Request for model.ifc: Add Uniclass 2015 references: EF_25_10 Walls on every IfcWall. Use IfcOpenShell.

First a look at what the model holds.

```python
import ifcopenshell

model = ifcopenshell.open("model.ifc")
print(model.schema)
print("classifications:", [c.Name for c in model.by_type("IfcClassification")])
for ifc_class in ("IfcDoor", "IfcRoof", "IfcStair", "IfcWall", "IfcWindow"):
    print(ifc_class, len(model.by_type(ifc_class)))
```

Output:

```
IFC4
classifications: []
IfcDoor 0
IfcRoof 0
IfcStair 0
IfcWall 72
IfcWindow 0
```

```python
import ifcopenshell
import ifcopenshell.api.classification

model = ifcopenshell.open("model.ifc")

system = ifcopenshell.api.classification.add_classification(model, classification="Uniclass 2015")

codes = {
    "IfcWall": ("EF_25_10", "Walls"),
}
for ifc_class, (code, name) in codes.items():
    products = model.by_type(ifc_class)
    ifcopenshell.api.classification.add_reference(
        model, products=products, classification=system, identification=code, name=name
    )
    print(code, len(products))

model.write("model_edited.ifc")
```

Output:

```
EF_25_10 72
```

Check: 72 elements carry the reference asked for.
